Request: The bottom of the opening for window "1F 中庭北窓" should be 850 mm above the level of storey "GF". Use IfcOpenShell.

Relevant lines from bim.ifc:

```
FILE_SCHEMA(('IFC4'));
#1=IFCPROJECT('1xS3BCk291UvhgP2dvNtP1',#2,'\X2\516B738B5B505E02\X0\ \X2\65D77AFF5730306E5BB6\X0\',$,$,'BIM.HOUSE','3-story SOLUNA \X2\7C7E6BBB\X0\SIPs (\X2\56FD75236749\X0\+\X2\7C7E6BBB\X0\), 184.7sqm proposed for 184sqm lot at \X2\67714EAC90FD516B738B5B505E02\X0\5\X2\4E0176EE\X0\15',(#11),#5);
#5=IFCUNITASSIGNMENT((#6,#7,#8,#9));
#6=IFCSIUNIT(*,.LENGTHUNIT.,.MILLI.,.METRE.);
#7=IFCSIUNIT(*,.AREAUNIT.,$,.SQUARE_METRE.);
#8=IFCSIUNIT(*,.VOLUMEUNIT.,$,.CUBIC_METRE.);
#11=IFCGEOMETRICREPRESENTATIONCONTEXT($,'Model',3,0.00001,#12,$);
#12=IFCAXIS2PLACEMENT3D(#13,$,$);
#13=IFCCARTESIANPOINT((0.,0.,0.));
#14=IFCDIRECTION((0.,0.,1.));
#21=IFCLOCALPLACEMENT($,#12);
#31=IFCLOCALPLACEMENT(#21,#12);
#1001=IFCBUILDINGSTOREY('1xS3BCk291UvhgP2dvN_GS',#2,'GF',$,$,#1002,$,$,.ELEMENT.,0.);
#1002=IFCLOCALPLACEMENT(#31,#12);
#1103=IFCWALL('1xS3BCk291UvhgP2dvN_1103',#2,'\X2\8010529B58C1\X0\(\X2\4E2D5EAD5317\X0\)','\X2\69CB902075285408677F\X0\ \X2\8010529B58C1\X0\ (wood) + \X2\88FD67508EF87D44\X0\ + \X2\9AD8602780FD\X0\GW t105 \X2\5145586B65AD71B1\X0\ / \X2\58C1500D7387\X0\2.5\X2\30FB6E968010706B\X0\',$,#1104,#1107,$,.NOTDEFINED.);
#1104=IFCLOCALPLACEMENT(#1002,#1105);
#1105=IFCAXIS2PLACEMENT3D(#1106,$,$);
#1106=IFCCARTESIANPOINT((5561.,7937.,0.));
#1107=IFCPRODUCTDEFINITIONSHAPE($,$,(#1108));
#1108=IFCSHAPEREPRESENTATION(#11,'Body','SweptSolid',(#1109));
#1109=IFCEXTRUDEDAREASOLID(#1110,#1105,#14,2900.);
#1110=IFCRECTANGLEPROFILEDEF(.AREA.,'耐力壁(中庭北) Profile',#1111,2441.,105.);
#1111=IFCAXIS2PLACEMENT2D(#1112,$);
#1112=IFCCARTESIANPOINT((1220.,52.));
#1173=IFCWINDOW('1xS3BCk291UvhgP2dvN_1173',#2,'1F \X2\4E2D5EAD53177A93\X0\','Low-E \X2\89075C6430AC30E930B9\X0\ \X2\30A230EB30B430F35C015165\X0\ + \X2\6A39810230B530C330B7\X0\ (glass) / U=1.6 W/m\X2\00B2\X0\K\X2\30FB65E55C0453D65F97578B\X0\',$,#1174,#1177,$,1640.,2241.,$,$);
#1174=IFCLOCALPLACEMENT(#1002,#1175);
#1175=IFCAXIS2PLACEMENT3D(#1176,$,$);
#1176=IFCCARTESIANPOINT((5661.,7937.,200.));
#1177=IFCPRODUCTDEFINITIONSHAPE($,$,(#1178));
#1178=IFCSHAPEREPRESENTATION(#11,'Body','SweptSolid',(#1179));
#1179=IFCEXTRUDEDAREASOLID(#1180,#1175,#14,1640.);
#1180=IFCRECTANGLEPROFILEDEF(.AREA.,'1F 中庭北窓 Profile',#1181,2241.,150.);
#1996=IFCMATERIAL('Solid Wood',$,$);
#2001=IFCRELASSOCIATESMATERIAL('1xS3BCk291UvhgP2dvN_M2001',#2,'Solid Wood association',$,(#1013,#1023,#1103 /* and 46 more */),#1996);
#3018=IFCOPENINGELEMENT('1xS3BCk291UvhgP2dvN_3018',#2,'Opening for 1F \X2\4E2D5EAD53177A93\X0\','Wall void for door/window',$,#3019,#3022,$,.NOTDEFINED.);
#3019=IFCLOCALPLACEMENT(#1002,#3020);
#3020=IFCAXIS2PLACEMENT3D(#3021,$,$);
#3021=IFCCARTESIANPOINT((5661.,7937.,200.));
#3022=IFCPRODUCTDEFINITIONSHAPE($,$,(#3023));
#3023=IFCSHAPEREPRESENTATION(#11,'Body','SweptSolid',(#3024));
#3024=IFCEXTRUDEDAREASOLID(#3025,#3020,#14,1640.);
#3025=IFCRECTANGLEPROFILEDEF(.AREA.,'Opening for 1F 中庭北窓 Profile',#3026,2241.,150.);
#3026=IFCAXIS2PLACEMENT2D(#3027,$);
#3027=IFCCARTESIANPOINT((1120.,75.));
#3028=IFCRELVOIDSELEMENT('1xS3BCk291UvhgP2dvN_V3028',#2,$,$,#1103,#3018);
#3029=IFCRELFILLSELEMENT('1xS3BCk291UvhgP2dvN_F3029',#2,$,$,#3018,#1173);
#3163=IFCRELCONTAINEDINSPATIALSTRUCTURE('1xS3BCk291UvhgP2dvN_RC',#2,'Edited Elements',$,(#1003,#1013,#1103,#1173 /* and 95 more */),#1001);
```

```python
import numpy as np
import ifcopenshell
import ifcopenshell.api.geometry
import ifcopenshell.geom
import ifcopenshell.util.element
import ifcopenshell.util.placement
import ifcopenshell.util.shape
import ifcopenshell.util.unit

model = ifcopenshell.open("bim.ifc")
unit_scale = ifcopenshell.util.unit.calculate_unit_scale(model)

window = model.by_id(1173)
opening = window.FillsVoids[0].RelatingOpeningElement
storey = ifcopenshell.util.element.get_container(window, ifc_class="IfcBuildingStorey")
level = ifcopenshell.util.placement.get_local_placement(storey.ObjectPlacement)[2, 3]

# The opening's origin need not be at the sill, so measure its lowest point.
shape = ifcopenshell.geom.create_shape(ifcopenshell.geom.settings(), opening)
bottom = ifcopenshell.util.shape.get_shape_bottom_elevation(shape, shape.geometry) / unit_scale
dz = level + 850.0 - bottom

shift = np.array([0.0, 0.0, dz])
# The window is not placed relative to its opening, so move both.
for product in (opening, window):
    matrix = ifcopenshell.util.placement.get_local_placement(product.ObjectPlacement)
    matrix[:3, 3] += shift
    ifcopenshell.api.geometry.edit_object_placement(model, product=product, matrix=matrix, is_si=False)

print(f"moved by {dz * unit_scale:+.3f} m")

model.write("bim_edited.ifc")
```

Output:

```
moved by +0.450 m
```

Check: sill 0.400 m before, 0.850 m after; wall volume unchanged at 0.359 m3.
